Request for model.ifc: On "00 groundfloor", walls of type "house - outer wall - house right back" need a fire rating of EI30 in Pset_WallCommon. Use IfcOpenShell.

First a look at what the model holds.

```python
import ifcopenshell
import ifcopenshell.util.element

model = ifcopenshell.open("model.ifc")
print(model.schema)
storey = next(s for s in model.by_type("IfcBuildingStorey") if s.Name == "00 groundfloor")
walls = [e for e in ifcopenshell.util.element.get_decomposition(storey) if e.is_a("IfcWall")]
seen = {}
for e in walls:
    element_type = ifcopenshell.util.element.get_type(e)
    key = (element_type.Name if element_type != e and element_type else None, ifcopenshell.util.element.get_pset(e, "Pset_WallCommon", "FireRating"))
    seen[key] = seen.get(key, 0) + 1
for (name, value), count in sorted(seen.items(), key=str):
    print(count, "x", name, "|", value)
```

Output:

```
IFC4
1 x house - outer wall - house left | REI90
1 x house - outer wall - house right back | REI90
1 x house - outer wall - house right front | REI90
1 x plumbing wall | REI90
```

```python
import ifcopenshell
import ifcopenshell.api.pset
import ifcopenshell.util.element

model = ifcopenshell.open("model.ifc")

storey = next(s for s in model.by_type("IfcBuildingStorey") if s.Name == "00 groundfloor")
walls = [e for e in ifcopenshell.util.element.get_decomposition(storey) if e.is_a("IfcWall")]

count = 0
for e in walls:
    element_type = ifcopenshell.util.element.get_type(e)
    if element_type in (None, e) or element_type.Name != "house - outer wall - house right back":
        continue
    # add_pset returns the element's existing set when there is one.
    pset = ifcopenshell.api.pset.add_pset(model, product=e, name="Pset_WallCommon")
    ifcopenshell.api.pset.edit_pset(model, pset=pset, properties={"FireRating": "EI30"})
    count += 1

print(count, "walls updated")

model.write("model-out.ifc")
```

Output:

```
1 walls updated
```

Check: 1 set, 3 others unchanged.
